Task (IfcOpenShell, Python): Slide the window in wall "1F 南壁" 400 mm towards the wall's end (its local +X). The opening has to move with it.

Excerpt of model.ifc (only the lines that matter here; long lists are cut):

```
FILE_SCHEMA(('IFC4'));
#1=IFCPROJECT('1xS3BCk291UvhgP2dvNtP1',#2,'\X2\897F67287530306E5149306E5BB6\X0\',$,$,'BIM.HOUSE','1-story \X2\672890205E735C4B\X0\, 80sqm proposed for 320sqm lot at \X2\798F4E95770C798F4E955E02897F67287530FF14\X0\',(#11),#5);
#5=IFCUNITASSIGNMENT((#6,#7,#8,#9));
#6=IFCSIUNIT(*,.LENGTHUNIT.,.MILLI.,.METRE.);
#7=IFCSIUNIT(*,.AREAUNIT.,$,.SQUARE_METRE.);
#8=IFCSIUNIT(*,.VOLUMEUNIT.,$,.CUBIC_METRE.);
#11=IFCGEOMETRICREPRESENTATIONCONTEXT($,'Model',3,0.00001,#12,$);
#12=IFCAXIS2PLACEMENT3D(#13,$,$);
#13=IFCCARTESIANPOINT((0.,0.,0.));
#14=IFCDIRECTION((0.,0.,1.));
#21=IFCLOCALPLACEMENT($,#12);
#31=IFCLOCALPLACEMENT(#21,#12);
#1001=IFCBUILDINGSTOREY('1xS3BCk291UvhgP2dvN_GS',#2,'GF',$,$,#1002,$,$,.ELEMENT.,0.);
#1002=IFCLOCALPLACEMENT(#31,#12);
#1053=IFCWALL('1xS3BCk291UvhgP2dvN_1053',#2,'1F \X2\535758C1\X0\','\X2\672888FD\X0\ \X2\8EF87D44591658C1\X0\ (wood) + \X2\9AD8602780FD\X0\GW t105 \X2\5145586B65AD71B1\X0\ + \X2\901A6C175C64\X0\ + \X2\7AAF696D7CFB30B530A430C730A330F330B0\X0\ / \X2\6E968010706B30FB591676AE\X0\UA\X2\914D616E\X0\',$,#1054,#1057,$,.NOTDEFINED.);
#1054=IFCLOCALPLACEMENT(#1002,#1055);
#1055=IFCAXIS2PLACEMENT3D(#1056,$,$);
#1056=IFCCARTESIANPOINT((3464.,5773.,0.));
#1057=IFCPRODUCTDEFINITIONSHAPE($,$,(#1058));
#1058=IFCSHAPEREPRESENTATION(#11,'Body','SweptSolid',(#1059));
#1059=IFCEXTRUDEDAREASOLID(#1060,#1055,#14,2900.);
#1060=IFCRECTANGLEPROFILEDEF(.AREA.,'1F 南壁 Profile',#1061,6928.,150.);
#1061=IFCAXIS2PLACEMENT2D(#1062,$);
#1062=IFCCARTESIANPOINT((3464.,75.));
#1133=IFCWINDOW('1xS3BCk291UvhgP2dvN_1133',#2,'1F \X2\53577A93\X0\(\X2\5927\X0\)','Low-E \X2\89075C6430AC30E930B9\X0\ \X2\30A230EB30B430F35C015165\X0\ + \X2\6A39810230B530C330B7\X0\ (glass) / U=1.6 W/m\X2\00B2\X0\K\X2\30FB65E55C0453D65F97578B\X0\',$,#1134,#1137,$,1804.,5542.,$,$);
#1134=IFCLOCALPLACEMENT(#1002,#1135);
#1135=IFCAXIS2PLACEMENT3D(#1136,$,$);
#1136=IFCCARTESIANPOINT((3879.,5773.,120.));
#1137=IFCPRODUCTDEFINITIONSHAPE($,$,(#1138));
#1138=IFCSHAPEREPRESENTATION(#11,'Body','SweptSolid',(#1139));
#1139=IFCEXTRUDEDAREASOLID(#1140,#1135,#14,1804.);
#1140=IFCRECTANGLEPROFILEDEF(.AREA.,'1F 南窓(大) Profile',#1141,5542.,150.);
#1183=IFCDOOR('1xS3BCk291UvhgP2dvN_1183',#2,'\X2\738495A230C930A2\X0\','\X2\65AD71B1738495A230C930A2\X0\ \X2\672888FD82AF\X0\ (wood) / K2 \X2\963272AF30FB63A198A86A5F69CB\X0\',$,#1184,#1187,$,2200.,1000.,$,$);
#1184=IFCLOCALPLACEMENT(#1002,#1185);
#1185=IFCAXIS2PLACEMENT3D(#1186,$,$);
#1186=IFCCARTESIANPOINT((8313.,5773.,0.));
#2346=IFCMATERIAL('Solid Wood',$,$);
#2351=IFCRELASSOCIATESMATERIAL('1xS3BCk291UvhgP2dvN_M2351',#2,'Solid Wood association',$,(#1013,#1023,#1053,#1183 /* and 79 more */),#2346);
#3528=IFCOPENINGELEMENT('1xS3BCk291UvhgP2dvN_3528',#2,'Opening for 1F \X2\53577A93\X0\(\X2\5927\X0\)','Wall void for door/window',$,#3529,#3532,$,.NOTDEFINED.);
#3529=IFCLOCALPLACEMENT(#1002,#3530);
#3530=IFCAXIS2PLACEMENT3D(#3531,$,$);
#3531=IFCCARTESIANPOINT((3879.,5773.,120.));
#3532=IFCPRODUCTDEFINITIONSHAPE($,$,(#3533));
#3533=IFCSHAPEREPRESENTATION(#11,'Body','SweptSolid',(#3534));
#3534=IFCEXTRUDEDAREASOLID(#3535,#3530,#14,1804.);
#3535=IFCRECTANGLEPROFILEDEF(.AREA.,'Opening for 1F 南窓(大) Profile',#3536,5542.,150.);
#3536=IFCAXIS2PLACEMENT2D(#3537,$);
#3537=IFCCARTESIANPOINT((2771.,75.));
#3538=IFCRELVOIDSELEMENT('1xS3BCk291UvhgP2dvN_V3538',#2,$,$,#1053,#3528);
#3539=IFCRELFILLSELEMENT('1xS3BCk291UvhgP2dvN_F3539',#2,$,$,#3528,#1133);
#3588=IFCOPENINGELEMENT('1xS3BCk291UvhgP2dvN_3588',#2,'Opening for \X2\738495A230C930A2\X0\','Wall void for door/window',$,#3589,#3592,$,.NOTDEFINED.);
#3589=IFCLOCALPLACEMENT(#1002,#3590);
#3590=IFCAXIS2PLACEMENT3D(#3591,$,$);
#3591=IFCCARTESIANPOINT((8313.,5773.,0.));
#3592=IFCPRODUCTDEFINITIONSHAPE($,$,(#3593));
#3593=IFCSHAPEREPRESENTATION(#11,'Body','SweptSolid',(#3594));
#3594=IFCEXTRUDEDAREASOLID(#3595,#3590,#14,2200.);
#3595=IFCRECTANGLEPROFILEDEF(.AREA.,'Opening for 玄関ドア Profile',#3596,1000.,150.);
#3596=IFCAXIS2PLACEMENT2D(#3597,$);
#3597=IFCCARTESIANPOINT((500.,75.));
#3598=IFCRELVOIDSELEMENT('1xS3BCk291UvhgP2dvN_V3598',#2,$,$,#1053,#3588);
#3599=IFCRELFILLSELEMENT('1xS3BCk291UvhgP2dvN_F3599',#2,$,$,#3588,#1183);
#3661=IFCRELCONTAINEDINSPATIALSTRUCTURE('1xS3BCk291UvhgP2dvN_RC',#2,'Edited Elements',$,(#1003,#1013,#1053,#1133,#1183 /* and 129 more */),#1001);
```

```python
import ifcopenshell
import ifcopenshell.api.geometry
import ifcopenshell.util.placement
import ifcopenshell.util.unit

model = ifcopenshell.open("model.ifc")
unit_scale = ifcopenshell.util.unit.calculate_unit_scale(model)

window = model.by_id(1133)
opening = window.FillsVoids[0].RelatingOpeningElement
wall = opening.VoidsElements[0].RelatingBuildingElement

wall_matrix = ifcopenshell.util.placement.get_local_placement(wall.ObjectPlacement)
shift = wall_matrix[:3, 0] * 0.4 / unit_scale
before = ifcopenshell.util.placement.get_local_placement(window.ObjectPlacement)[:3, 3].copy()

# The window is not placed relative to its opening, so move both.
for product in (opening, window):
    matrix = ifcopenshell.util.placement.get_local_placement(product.ObjectPlacement)
    matrix[:3, 3] += shift
    ifcopenshell.api.geometry.edit_object_placement(model, product=product, matrix=matrix, is_si=False)

after = ifcopenshell.util.placement.get_local_placement(window.ObjectPlacement)[:3, 3]
print("window moved by", (after - before).round(3) + 0.0)

model.write("model_v2.ifc")
```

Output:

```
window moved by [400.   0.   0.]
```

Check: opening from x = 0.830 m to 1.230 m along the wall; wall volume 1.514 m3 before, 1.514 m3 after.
